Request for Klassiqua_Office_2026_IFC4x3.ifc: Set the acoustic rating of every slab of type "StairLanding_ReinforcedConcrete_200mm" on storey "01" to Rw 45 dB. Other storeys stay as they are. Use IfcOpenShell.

First a look at what the model holds.

```python
import ifcopenshell
import ifcopenshell.util.element

model = ifcopenshell.open("Klassiqua_Office_2026_IFC4x3.ifc")
print(model.schema)
storey = next(s for s in model.by_type("IfcBuildingStorey") if s.Name == "01")
slabs = [e for e in ifcopenshell.util.element.get_decomposition(storey) if e.is_a("IfcSlab")]
seen = {}
for e in slabs:
    element_type = ifcopenshell.util.element.get_type(e)
    key = (element_type.Name if element_type != e and element_type else None, ifcopenshell.util.element.get_pset(e, "Pset_SlabCommon", "AcousticRating"))
    seen[key] = seen.get(key, 0) + 1
for (name, value), count in sorted(seen.items(), key=str):
    print(count, "x", name, "|", value)
```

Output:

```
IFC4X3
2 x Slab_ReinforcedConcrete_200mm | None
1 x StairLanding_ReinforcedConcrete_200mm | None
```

```python
import ifcopenshell
import ifcopenshell.api.pset
import ifcopenshell.util.element

model = ifcopenshell.open("Klassiqua_Office_2026_IFC4x3.ifc")

storey = next(s for s in model.by_type("IfcBuildingStorey") if s.Name == "01")
slabs = [e for e in ifcopenshell.util.element.get_decomposition(storey) if e.is_a("IfcSlab")]

count = 0
for e in slabs:
    element_type = ifcopenshell.util.element.get_type(e)
    if element_type in (None, e) or element_type.Name != "StairLanding_ReinforcedConcrete_200mm":
        continue
    # add_pset returns the element's existing set when there is one.
    pset = ifcopenshell.api.pset.add_pset(model, product=e, name="Pset_SlabCommon")
    ifcopenshell.api.pset.edit_pset(model, pset=pset, properties={"AcousticRating": "Rw 45 dB"})
    count += 1

print(count, "slabs updated")

model.write("Klassiqua_Office_2026_IFC4x3_rev.ifc")
```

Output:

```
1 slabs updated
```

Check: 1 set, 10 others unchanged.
